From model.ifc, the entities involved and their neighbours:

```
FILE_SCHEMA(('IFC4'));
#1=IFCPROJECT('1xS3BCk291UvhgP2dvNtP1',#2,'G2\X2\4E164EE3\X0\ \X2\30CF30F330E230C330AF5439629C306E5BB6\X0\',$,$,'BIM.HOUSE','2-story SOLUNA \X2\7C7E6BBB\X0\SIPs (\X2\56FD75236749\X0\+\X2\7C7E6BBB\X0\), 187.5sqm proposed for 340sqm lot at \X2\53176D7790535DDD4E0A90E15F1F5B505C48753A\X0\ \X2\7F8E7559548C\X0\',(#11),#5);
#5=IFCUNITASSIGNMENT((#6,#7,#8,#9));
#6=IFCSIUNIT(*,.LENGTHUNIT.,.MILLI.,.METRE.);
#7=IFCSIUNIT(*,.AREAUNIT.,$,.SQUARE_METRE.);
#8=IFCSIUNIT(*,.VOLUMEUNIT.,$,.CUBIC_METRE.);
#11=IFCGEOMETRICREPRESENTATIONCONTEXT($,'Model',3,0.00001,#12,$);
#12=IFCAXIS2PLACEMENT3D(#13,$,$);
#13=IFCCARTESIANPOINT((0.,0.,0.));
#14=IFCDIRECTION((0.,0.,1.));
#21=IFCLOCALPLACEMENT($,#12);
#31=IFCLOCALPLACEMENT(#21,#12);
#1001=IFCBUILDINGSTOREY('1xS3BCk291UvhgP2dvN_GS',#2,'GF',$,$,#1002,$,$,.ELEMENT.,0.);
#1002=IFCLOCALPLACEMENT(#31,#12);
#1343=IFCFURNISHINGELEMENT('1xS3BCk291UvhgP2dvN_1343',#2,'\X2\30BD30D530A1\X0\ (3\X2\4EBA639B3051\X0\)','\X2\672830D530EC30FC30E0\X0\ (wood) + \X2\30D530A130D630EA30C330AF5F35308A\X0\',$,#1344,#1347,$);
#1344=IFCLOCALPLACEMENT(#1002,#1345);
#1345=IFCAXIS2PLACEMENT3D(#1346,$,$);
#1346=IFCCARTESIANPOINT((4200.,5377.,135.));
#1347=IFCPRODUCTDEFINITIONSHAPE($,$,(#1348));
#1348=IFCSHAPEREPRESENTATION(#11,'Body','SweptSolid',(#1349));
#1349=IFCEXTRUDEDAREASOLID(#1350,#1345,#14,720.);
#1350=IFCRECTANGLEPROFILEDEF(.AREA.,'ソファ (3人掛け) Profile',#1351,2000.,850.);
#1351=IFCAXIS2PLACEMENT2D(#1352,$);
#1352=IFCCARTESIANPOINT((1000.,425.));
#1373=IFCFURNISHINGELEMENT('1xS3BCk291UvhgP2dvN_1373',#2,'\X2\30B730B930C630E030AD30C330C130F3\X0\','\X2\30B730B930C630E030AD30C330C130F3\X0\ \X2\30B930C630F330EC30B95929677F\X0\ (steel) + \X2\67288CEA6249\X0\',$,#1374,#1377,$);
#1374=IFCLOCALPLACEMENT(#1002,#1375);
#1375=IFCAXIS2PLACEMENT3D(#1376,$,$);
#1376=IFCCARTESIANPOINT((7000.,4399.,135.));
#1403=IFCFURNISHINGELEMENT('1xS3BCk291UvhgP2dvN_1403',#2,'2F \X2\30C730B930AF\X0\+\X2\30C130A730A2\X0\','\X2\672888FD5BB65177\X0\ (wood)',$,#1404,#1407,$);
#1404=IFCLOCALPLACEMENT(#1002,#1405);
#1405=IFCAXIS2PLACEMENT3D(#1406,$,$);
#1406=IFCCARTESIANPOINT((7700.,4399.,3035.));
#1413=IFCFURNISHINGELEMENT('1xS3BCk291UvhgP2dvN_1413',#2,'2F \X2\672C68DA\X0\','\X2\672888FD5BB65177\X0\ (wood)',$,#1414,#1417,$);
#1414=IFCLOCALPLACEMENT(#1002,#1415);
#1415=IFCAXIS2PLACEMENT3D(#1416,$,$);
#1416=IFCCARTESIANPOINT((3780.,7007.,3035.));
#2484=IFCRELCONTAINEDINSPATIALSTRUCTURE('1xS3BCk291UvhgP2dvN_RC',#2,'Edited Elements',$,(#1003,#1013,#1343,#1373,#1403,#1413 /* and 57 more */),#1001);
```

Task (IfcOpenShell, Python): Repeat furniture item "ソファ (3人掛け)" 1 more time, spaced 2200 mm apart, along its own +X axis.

```python
import ifcopenshell
import ifcopenshell.api.geometry
import ifcopenshell.api.root
import ifcopenshell.util.element
import ifcopenshell.util.placement
import ifcopenshell.util.unit

model = ifcopenshell.open("model.ifc")
unit_scale = ifcopenshell.util.unit.calculate_unit_scale(model)


def reuse_history(source, copy):
    """copy_class also copies each property set's owner history, people and application; keep the originals."""
    for rel in copy.IsDefinedBy:
        if rel.is_a("IfcRelDefinesByProperties") and (history := rel.RelatingPropertyDefinition.OwnerHistory):
            rel.RelatingPropertyDefinition.OwnerHistory = source.OwnerHistory
            ifcopenshell.util.element.remove_deep2(model, history)


source = model.by_guid("1xS3BCk291UvhgP2dvN_1343")
base = ifcopenshell.util.placement.get_local_placement(source.ObjectPlacement)
step = base[:3, 0] * 2.2 / unit_scale

for i in range(1, 2):
    copy = ifcopenshell.api.root.copy_class(model, product=source)
    copy.Representation = ifcopenshell.util.element.copy_deep(
        model, source.Representation, exclude=["IfcGeometricRepresentationContext", "IfcRepresentationMap"]
    )
    reuse_history(source, copy)
    matrix = base.copy()
    matrix[:3, 3] += i * step
    print("added at", matrix[:3, 3].round(3) + 0.0)
    ifcopenshell.api.geometry.edit_object_placement(model, product=copy, matrix=matrix, is_si=False)

model.write("model-out.ifc")
```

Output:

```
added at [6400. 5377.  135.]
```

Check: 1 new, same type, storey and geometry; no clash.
